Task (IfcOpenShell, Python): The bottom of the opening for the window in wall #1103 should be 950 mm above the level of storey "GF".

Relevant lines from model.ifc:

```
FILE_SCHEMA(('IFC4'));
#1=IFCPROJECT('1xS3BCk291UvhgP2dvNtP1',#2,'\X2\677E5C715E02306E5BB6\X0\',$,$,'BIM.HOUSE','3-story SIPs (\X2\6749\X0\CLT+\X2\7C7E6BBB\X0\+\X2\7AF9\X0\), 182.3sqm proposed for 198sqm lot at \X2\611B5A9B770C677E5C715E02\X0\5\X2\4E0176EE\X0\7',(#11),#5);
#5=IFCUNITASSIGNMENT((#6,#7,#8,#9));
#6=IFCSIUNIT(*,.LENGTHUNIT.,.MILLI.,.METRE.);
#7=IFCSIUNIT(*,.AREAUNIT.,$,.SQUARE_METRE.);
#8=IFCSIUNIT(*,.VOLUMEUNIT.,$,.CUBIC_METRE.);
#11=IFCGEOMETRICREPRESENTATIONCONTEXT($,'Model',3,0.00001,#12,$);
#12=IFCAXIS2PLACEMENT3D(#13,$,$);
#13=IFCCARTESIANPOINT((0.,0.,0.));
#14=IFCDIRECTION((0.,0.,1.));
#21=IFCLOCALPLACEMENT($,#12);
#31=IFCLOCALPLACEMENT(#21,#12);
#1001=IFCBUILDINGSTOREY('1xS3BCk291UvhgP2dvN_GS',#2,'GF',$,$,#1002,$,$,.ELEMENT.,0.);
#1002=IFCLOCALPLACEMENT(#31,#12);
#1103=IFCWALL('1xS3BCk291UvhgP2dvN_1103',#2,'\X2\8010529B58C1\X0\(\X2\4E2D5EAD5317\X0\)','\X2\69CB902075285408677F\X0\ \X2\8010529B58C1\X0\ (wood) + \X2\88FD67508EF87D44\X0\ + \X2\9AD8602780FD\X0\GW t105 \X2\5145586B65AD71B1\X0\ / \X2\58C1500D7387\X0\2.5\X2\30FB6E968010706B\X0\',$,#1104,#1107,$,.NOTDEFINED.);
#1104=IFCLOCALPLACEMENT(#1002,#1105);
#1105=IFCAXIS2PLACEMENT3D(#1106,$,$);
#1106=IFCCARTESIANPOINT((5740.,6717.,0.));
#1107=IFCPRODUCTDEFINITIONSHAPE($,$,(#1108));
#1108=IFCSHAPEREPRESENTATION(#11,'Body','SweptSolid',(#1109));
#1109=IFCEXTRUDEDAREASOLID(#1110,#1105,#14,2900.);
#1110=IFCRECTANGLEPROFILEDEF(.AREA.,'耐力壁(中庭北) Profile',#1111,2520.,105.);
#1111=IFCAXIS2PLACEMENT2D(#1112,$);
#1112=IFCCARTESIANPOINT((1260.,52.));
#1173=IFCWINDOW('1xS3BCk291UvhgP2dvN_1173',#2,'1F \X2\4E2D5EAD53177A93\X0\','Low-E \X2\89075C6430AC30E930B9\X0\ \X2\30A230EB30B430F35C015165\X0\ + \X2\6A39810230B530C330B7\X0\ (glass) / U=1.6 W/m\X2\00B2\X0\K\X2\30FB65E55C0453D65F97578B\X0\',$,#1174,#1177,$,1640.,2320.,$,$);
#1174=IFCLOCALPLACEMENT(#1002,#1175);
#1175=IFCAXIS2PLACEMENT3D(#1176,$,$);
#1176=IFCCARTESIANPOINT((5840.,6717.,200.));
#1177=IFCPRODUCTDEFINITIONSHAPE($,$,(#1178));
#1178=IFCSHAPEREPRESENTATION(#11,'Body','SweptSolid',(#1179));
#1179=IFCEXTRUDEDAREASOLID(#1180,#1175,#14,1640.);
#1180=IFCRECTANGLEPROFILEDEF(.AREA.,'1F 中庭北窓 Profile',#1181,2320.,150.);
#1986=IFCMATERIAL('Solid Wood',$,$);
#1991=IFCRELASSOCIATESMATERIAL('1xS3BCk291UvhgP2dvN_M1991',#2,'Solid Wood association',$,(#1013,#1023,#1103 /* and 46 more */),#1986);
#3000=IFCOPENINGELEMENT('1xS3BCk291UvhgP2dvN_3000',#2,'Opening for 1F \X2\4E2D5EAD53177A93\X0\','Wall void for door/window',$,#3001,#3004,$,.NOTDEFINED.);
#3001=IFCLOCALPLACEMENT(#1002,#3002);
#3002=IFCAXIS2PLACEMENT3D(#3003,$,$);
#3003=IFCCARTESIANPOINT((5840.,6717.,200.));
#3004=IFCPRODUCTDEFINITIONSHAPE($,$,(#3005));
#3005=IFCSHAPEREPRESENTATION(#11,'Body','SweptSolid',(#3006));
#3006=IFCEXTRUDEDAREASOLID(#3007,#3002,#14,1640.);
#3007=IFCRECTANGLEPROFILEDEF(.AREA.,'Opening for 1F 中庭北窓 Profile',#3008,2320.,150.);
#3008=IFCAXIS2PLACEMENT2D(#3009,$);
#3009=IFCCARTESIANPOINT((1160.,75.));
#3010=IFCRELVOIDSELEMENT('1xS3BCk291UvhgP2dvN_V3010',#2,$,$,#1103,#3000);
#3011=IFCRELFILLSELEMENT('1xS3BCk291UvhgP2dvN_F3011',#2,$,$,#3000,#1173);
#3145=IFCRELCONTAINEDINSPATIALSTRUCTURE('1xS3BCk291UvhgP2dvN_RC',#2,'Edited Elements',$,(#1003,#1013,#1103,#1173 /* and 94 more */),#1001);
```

```python
import numpy as np
import ifcopenshell
import ifcopenshell.api.geometry
import ifcopenshell.geom
import ifcopenshell.util.element
import ifcopenshell.util.placement
import ifcopenshell.util.shape
import ifcopenshell.util.unit

model = ifcopenshell.open("model.ifc")
unit_scale = ifcopenshell.util.unit.calculate_unit_scale(model)

window = model.by_guid("1xS3BCk291UvhgP2dvN_1173")
opening = window.FillsVoids[0].RelatingOpeningElement
storey = ifcopenshell.util.element.get_container(window, ifc_class="IfcBuildingStorey")
level = ifcopenshell.util.placement.get_local_placement(storey.ObjectPlacement)[2, 3]

# The opening's origin need not be at the sill, so measure its lowest point.
shape = ifcopenshell.geom.create_shape(ifcopenshell.geom.settings(), opening)
bottom = ifcopenshell.util.shape.get_shape_bottom_elevation(shape, shape.geometry) / unit_scale
dz = level + 0.95 / unit_scale - bottom

shift = np.array([0.0, 0.0, dz])
# The window is not placed relative to its opening, so move both.
for product in (opening, window):
    matrix = ifcopenshell.util.placement.get_local_placement(product.ObjectPlacement)
    matrix[:3, 3] += shift
    ifcopenshell.api.geometry.edit_object_placement(model, product=product, matrix=matrix, is_si=False)

print(f"moved by {dz * unit_scale:+.3f} m")

model.write("model_updated.ifc")
```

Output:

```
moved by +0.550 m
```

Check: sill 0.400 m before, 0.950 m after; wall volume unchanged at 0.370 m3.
